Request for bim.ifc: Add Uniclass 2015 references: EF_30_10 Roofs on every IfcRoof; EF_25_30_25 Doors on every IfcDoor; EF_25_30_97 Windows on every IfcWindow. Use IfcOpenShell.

First a look at what the model holds.

```python
import ifcopenshell

model = ifcopenshell.open("bim.ifc")
print(model.schema)
print("classifications:", [c.Name for c in model.by_type("IfcClassification")])
for ifc_class in ("IfcDoor", "IfcRoof", "IfcStair", "IfcWall", "IfcWindow"):
    print(ifc_class, len(model.by_type(ifc_class)))
```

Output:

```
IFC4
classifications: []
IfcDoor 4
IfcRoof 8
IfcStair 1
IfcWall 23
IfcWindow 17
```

```python
import ifcopenshell
import ifcopenshell.api.classification

model = ifcopenshell.open("bim.ifc")

system = ifcopenshell.api.classification.add_classification(model, classification="Uniclass 2015")

codes = {
    "IfcRoof": ("EF_30_10", "Roofs"),
    "IfcDoor": ("EF_25_30_25", "Doors"),
    "IfcWindow": ("EF_25_30_97", "Windows"),
}
for ifc_class, (code, name) in codes.items():
    products = model.by_type(ifc_class)
    ifcopenshell.api.classification.add_reference(
        model, products=products, classification=system, identification=code, name=name
    )
    print(code, len(products))

model.write("bim-out.ifc")
```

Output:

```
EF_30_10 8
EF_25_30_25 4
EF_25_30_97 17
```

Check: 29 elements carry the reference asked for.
